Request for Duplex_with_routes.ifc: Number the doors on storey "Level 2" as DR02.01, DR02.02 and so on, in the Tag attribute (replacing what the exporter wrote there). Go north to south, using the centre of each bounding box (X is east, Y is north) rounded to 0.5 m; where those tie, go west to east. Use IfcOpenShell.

First a look at what the model holds.

```python
import ifcopenshell
import ifcopenshell.util.element
import ifcopenshell.util.placement

model = ifcopenshell.open("Duplex_with_routes.ifc")
print(model.schema)
storey = next(s for s in model.by_type("IfcBuildingStorey") if s.Name == "Level 2")
doors = [e for e in ifcopenshell.util.element.get_decomposition(storey) if e.is_a("IfcDoor")]
for e in sorted(doors, key=lambda e: e.id()):
    origin = ifcopenshell.util.placement.get_local_placement(e.ObjectPlacement)[:3, 3]
    print(e.id(), e.Tag, e.Name, origin.round(2) + 0.0, sep=" | ")
```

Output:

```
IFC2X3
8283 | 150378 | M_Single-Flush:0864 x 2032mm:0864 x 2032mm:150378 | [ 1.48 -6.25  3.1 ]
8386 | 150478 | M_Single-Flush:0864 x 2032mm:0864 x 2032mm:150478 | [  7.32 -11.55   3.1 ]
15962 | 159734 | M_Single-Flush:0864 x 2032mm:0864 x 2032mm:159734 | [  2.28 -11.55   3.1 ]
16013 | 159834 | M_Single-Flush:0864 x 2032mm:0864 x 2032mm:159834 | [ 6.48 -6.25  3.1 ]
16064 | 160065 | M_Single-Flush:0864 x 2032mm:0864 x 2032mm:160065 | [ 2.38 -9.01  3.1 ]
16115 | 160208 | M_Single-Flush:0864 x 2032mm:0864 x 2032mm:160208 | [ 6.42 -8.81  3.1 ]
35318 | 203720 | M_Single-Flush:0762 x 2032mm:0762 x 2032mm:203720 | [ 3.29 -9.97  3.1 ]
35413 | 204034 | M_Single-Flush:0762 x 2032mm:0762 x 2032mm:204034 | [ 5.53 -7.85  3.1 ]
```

```python
import ifcopenshell
import ifcopenshell.geom
import ifcopenshell.util.element
import ifcopenshell.util.shape

model = ifcopenshell.open("Duplex_with_routes.ifc")
settings = ifcopenshell.geom.settings()
settings.set("use-world-coords", True)


def centre(element):
    shape = ifcopenshell.geom.create_shape(settings, element)
    return ifcopenshell.util.shape.get_bbox_centroid(shape.geometry)


storey = next(s for s in model.by_type("IfcBuildingStorey") if s.Name == "Level 2")
doors = [e for e in ifcopenshell.util.element.get_decomposition(storey) if e.is_a("IfcDoor")]

# Insertion points can sit at a corner or the storey origin, so sort by the geometry (in metres).
centres = {e: centre(e) for e in doors}
doors.sort(key=lambda e: (-round(centres[e][1] / 0.5), centres[e][0]))

for i, e in enumerate(doors, start=1):
    number = f"DR02.{i:02d}"
    e.Tag = number
    print(e.id(), number)

model.write("Duplex_with_routes_rev.ifc")
```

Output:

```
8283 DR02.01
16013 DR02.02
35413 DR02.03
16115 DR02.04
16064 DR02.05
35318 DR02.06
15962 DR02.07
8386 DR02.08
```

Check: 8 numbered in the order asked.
